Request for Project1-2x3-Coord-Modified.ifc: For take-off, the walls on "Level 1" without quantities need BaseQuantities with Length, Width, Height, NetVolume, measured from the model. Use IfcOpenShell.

First a look at what the model holds.

```python
import ifcopenshell
import ifcopenshell.util.element
import ifcopenshell.util.unit

model = ifcopenshell.open("Project1-2x3-Coord-Modified.ifc")
print(model.schema)
for unit_type in ("LENGTHUNIT", "AREAUNIT", "VOLUMEUNIT"):
    print(unit_type, ifcopenshell.util.unit.calculate_unit_scale(model, unit_type))
storey = next(s for s in model.by_type("IfcBuildingStorey") if s.Name == "Level 1")
walls = [e for e in ifcopenshell.util.element.get_decomposition(storey) if e.is_a("IfcWall")]
for e in sorted(walls, key=lambda e: e.id()):
    print(e.id(), e.is_a(), e.Name, list(ifcopenshell.util.element.get_psets(e, qtos_only=True)), sep=" | ")
```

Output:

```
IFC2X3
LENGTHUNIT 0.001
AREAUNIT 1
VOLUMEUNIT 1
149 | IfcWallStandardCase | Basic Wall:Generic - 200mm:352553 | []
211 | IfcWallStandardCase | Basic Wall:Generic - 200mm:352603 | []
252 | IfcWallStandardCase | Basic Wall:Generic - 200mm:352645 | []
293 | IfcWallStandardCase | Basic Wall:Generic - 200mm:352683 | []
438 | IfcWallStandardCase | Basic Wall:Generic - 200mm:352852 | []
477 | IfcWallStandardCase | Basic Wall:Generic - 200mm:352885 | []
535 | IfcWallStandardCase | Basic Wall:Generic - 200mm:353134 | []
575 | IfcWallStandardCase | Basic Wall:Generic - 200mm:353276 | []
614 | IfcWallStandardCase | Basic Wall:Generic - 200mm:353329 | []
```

```python
import ifcopenshell
import ifcopenshell.api.pset
import ifcopenshell.geom
import ifcopenshell.util.element
import ifcopenshell.util.shape
import ifcopenshell.util.unit

model = ifcopenshell.open("Project1-2x3-Coord-Modified.ifc")
unit_scale = ifcopenshell.util.unit.calculate_unit_scale(model)
volume_scale = ifcopenshell.util.unit.calculate_unit_scale(model, "VOLUMEUNIT")
settings = ifcopenshell.geom.settings()

storey = next(s for s in model.by_type("IfcBuildingStorey") if s.Name == "Level 1")
walls = [e for e in ifcopenshell.util.element.get_decomposition(storey) if e.is_a("IfcWall")]

for e in sorted(walls, key=lambda e: e.id()):
    if ifcopenshell.util.element.get_psets(e, qtos_only=True, should_inherit=False):
        continue
    # Geometry comes back in metres, in the element's own axes.
    shape = ifcopenshell.geom.create_shape(settings, e)
    values = {
        "Length": ifcopenshell.util.shape.get_x(shape.geometry) / unit_scale,
        "Width": ifcopenshell.util.shape.get_y(shape.geometry) / unit_scale,
        "Height": ifcopenshell.util.shape.get_z(shape.geometry) / unit_scale,
        "NetVolume": ifcopenshell.util.shape.get_volume(shape.geometry) / volume_scale,
    }
    qto = ifcopenshell.api.pset.add_qto(model, product=e, name="BaseQuantities")
    ifcopenshell.api.pset.edit_qto(model, qto=qto, properties=values)
    print(e.id(), {k: round(v, 3) for k, v in values.items()})

model.write("Project1-2x3-Coord-Modified-out.ifc")
```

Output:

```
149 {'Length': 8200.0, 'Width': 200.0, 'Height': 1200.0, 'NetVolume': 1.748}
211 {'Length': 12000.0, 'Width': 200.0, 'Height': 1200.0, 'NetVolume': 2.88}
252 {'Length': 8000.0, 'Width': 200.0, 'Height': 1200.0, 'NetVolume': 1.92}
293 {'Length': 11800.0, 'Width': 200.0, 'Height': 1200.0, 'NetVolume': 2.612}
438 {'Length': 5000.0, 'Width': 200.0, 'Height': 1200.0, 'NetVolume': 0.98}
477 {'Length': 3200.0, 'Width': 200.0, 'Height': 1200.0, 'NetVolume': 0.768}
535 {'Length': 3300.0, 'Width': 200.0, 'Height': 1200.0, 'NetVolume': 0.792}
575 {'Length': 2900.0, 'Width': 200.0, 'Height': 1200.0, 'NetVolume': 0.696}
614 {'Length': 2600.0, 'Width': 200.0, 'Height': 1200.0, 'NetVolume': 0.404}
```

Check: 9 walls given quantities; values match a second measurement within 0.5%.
